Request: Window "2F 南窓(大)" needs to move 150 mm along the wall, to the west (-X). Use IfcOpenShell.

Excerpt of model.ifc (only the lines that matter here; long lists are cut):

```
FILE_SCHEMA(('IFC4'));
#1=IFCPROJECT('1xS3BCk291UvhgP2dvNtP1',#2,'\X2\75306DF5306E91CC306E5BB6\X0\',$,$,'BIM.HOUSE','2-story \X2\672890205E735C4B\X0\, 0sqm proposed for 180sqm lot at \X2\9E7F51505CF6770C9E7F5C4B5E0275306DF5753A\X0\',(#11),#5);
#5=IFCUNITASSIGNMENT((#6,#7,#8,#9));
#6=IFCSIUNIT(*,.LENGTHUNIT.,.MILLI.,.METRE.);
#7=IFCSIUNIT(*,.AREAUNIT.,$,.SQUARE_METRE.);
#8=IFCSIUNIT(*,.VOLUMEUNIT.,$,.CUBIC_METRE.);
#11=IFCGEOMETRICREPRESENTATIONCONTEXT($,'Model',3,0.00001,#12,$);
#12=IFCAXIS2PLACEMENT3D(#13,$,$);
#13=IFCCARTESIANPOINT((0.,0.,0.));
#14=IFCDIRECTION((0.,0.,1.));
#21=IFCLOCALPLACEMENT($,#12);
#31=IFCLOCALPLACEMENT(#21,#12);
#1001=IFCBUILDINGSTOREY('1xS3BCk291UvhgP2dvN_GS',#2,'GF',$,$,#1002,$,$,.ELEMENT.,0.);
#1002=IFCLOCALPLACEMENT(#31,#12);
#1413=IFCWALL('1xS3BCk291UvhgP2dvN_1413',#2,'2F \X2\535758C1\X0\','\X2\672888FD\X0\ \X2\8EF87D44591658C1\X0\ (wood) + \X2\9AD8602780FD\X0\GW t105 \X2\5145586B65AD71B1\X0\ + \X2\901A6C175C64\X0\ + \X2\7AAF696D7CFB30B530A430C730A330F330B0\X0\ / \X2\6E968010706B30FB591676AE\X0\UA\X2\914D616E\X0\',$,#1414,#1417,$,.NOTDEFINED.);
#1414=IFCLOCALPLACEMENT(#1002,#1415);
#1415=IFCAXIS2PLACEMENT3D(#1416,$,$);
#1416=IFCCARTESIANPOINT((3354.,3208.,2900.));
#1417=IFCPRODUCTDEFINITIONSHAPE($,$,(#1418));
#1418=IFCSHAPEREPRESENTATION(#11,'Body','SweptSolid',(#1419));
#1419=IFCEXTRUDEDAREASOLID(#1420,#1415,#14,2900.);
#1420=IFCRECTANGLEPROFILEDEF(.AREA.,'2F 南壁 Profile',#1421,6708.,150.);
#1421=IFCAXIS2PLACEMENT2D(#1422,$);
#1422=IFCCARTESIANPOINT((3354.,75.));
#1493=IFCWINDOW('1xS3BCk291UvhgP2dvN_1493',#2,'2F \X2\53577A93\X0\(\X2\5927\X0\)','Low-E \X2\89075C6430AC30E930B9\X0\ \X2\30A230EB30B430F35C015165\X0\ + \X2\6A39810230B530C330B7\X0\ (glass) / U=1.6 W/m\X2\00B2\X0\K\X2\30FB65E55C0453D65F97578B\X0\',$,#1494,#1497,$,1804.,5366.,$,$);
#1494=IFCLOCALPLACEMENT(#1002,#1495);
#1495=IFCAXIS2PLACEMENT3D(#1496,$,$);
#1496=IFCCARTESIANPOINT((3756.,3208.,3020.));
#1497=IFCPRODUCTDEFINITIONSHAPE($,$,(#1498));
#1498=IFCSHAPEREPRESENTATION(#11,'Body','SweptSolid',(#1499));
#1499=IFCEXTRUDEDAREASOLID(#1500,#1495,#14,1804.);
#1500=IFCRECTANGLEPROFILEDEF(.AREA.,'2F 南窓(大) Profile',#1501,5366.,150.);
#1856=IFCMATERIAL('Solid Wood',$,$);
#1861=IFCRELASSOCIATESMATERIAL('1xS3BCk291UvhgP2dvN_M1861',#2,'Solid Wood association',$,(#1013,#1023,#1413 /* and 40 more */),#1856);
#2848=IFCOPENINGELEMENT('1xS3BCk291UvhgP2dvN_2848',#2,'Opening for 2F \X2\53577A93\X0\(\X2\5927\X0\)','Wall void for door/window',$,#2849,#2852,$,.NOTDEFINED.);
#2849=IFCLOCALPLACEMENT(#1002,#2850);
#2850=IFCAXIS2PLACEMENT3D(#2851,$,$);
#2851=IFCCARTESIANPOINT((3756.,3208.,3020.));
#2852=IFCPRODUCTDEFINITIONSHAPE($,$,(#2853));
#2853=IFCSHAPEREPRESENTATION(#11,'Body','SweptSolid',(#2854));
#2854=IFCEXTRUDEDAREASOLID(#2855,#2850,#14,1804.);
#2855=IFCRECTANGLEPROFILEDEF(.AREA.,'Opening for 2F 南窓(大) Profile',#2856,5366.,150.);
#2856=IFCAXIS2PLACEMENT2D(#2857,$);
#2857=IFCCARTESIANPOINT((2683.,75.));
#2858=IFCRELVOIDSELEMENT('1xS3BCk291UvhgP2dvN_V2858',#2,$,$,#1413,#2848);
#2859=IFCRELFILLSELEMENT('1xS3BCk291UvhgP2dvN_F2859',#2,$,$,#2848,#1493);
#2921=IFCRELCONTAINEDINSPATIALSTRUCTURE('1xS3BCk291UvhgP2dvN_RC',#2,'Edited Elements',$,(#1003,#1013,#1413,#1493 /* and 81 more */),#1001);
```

```python
import ifcopenshell
import ifcopenshell.api.geometry
import ifcopenshell.util.placement
import ifcopenshell.util.unit

model = ifcopenshell.open("model.ifc")
unit_scale = ifcopenshell.util.unit.calculate_unit_scale(model)

window = model.by_guid("1xS3BCk291UvhgP2dvN_1493")
opening = window.FillsVoids[0].RelatingOpeningElement
wall = opening.VoidsElements[0].RelatingBuildingElement

wall_matrix = ifcopenshell.util.placement.get_local_placement(wall.ObjectPlacement)
shift = wall_matrix[:3, 0] * -0.15 / unit_scale
before = ifcopenshell.util.placement.get_local_placement(window.ObjectPlacement)[:3, 3].copy()

# The window is not placed relative to its opening, so move both.
for product in (opening, window):
    matrix = ifcopenshell.util.placement.get_local_placement(product.ObjectPlacement)
    matrix[:3, 3] += shift
    ifcopenshell.api.geometry.edit_object_placement(model, product=product, matrix=matrix, is_si=False)

after = ifcopenshell.util.placement.get_local_placement(window.ObjectPlacement)[:3, 3]
print("window moved by", (after - before).round(3) + 0.0)

model.write("model-out.ifc")
```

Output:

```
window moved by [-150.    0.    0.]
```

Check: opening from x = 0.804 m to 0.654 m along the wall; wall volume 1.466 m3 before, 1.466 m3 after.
